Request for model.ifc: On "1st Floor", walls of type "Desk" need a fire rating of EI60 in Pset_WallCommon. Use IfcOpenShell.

First a look at what the model holds.

```python
import ifcopenshell
import ifcopenshell.util.element

model = ifcopenshell.open("model.ifc")
print(model.schema)
storey = next(s for s in model.by_type("IfcBuildingStorey") if s.Name == "1st Floor")
walls = [e for e in ifcopenshell.util.element.get_decomposition(storey) if e.is_a("IfcWall")]
seen = {}
for e in walls:
    element_type = ifcopenshell.util.element.get_type(e)
    key = (element_type.Name if element_type != e and element_type else None, ifcopenshell.util.element.get_pset(e, "Pset_WallCommon", "FireRating"))
    seen[key] = seen.get(key, 0) + 1
for (name, value), count in sorted(seen.items(), key=str):
    print(count, "x", name, "|", value)
```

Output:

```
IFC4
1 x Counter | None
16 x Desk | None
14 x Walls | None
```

```python
import ifcopenshell
import ifcopenshell.api.pset
import ifcopenshell.util.element

model = ifcopenshell.open("model.ifc")

storey = next(s for s in model.by_type("IfcBuildingStorey") if s.Name == "1st Floor")
walls = [e for e in ifcopenshell.util.element.get_decomposition(storey) if e.is_a("IfcWall")]

count = 0
for e in walls:
    element_type = ifcopenshell.util.element.get_type(e)
    if element_type in (None, e) or element_type.Name != "Desk":
        continue
    # add_pset returns the element's existing set when there is one.
    pset = ifcopenshell.api.pset.add_pset(model, product=e, name="Pset_WallCommon")
    ifcopenshell.api.pset.edit_pset(model, pset=pset, properties={"FireRating": "EI60"})
    count += 1

print(count, "walls updated")

model.write("model_rev.ifc")
```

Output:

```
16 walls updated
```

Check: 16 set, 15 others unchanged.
